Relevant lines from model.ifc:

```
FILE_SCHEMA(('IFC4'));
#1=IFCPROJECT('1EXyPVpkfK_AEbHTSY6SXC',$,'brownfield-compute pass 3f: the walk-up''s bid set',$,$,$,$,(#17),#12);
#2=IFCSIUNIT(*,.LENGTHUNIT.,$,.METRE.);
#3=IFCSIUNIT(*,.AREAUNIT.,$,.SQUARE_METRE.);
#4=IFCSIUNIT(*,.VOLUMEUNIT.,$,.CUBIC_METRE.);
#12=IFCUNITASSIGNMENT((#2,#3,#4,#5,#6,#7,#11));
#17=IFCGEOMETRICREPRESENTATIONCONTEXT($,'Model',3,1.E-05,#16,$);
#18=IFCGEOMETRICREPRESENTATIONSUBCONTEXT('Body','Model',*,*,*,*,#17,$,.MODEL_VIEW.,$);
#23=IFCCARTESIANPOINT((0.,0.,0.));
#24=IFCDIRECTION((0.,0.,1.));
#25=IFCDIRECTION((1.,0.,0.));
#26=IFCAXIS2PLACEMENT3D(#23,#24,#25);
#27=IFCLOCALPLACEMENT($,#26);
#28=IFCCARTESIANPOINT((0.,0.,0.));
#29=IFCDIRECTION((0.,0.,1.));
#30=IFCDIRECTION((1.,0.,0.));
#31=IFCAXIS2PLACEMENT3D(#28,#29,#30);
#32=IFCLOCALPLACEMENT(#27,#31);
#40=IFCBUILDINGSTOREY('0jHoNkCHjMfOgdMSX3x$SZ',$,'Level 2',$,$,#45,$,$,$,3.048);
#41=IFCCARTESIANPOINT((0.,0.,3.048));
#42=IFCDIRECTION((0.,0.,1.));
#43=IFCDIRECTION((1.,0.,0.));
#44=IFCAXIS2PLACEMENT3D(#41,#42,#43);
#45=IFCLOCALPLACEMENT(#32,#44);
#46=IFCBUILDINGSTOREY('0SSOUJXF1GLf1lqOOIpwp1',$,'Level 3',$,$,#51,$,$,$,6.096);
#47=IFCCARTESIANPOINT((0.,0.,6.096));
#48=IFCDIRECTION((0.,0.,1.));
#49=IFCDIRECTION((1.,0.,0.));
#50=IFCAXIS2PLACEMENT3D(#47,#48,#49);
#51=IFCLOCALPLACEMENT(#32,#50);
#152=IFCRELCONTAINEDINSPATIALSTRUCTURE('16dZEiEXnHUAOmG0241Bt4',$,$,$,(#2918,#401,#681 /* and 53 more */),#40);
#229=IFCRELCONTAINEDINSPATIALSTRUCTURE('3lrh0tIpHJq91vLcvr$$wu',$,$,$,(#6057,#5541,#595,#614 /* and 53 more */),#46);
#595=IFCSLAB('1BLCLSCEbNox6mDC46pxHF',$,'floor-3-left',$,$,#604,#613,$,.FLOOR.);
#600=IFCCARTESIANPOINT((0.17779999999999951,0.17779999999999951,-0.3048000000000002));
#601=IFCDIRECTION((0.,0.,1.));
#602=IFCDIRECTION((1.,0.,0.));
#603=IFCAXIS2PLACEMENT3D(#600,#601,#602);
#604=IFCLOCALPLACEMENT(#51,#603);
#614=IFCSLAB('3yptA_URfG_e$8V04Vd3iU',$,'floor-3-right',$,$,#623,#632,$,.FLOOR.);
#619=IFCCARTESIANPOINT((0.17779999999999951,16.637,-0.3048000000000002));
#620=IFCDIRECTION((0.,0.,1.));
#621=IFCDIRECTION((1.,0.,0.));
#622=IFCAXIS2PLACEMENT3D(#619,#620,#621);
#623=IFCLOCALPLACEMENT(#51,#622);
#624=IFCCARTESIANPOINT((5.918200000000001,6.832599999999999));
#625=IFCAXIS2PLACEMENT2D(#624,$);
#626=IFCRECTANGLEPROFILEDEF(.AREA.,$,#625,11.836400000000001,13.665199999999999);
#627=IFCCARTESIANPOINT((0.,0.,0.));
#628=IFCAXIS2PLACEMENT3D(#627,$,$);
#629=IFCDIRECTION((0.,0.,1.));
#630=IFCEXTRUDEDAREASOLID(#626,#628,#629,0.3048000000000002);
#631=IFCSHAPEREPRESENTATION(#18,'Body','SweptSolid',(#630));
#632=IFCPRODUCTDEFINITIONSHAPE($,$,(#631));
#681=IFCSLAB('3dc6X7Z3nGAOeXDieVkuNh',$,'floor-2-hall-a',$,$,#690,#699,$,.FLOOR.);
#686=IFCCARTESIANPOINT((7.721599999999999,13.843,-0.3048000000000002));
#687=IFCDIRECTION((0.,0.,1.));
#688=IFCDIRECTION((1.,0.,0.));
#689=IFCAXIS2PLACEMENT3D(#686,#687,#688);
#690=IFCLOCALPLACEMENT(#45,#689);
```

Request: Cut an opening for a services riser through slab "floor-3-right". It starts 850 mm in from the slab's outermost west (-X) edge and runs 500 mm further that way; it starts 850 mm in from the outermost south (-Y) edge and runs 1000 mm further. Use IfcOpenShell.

```python
import numpy as np
import ifcopenshell
import ifcopenshell.api.feature
import ifcopenshell.api.geometry
import ifcopenshell.api.root
import ifcopenshell.geom
import ifcopenshell.util.placement
import ifcopenshell.util.representation
import ifcopenshell.util.shape
import ifcopenshell.util.unit

model = ifcopenshell.open("model.ifc")
unit_scale = ifcopenshell.util.unit.calculate_unit_scale(model)
settings = ifcopenshell.geom.settings()


def volume(element):
    """Net volume in cubic metres, openings subtracted."""
    shape = ifcopenshell.geom.create_shape(settings, element)
    return ifcopenshell.util.shape.get_volume(shape.geometry)


slab = model.by_guid("3yptA_URfG_e$8V04Vd3iU")
before = volume(slab)

# Extent in the slab's own axes, in metres. The edges named are its -X and -Y sides.
slab_shape = ifcopenshell.geom.create_shape(settings, slab)
vertices = ifcopenshell.util.shape.get_vertices(slab_shape.geometry)
x_min, y_min, bottom = vertices.min(axis=0)
top = vertices[:, 2].max()

opening = ifcopenshell.api.root.create_entity(model, ifc_class="IfcOpeningElement", name="Services riser opening", predefined_type="OPENING")
context = ifcopenshell.util.representation.get_context(model, "Model", "Body", "MODEL_VIEW")
width, depth = 0.5, 1
outline = [(0.0, 0.0), (width, 0.0), (width, depth), (0.0, depth), (0.0, 0.0)]
# Overshoot both faces by 50 mm so the cut is clean.
shape = ifcopenshell.api.geometry.add_slab_representation(
    model, context=context, depth=top - bottom + 0.1, polyline=outline
)
ifcopenshell.api.geometry.assign_representation(model, product=opening, representation=shape)

matrix = ifcopenshell.util.placement.get_local_placement(slab.ObjectPlacement)
matrix[:, 3] = matrix @ np.append(np.array([x_min + 0.85, y_min + 0.85, bottom - 0.05]) / unit_scale, 1.0)
ifcopenshell.api.geometry.edit_object_placement(model, product=opening, matrix=matrix, is_si=False)
ifcopenshell.api.feature.add_feature(model, feature=opening, element=slab)

after = volume(slab)

print(f"slab volume {before:.3f} -> {after:.3f} m3")

model.write("model_edited.ifc")
```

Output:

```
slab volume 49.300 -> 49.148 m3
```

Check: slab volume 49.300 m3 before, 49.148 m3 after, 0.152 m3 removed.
